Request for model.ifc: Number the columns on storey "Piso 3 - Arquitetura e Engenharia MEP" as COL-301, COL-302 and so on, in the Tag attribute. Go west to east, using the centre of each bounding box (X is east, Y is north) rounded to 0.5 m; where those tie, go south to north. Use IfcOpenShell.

First a look at what the model holds.

```python
import ifcopenshell
import ifcopenshell.util.element
import ifcopenshell.util.placement

model = ifcopenshell.open("model.ifc")
print(model.schema)
storey = next(s for s in model.by_type("IfcBuildingStorey") if s.Name == "Piso 3 - Arquitetura e Engenharia MEP")
columns = [e for e in ifcopenshell.util.element.get_decomposition(storey) if e.is_a("IfcColumn")]
for e in sorted(columns, key=lambda e: e.id()):
    origin = ifcopenshell.util.placement.get_local_placement(e.ObjectPlacement)[:3, 3]
    print(e.id(), e.Tag, e.Name, origin.round(2) + 0.0, sep=" | ")
```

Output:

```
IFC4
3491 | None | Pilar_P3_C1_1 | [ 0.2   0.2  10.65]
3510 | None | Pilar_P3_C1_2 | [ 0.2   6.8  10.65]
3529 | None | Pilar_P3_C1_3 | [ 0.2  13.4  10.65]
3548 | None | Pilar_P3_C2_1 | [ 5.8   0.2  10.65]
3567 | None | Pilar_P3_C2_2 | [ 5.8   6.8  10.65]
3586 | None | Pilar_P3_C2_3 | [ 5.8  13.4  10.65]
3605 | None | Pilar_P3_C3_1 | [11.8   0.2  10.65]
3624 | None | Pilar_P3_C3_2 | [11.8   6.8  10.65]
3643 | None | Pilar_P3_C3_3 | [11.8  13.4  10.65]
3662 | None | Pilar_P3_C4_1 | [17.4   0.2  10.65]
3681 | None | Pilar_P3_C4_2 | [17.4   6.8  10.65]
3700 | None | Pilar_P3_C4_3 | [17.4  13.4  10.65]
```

```python
import ifcopenshell
import ifcopenshell.geom
import ifcopenshell.util.element
import ifcopenshell.util.shape

model = ifcopenshell.open("model.ifc")
settings = ifcopenshell.geom.settings()
settings.set("use-world-coords", True)


def centre(element):
    shape = ifcopenshell.geom.create_shape(settings, element)
    return ifcopenshell.util.shape.get_bbox_centroid(shape.geometry)


storey = next(s for s in model.by_type("IfcBuildingStorey") if s.Name == "Piso 3 - Arquitetura e Engenharia MEP")
columns = [e for e in ifcopenshell.util.element.get_decomposition(storey) if e.is_a("IfcColumn")]

# Insertion points can sit at a corner or the storey origin, so sort by the geometry (in metres).
centres = {e: centre(e) for e in columns}
columns.sort(key=lambda e: (round(centres[e][0] / 0.5), centres[e][1]))

for i, e in enumerate(columns, start=1):
    number = f"COL-3{i:02d}"
    e.Tag = number
    print(e.id(), number)

model.write("model-out.ifc")
```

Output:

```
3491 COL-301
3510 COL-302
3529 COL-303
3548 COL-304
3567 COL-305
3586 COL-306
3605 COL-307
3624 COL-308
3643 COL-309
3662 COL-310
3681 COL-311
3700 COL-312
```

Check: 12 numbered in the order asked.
